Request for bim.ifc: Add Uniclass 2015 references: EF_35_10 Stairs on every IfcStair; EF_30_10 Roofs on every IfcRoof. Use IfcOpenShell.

First a look at what the model holds.

```python
import ifcopenshell

model = ifcopenshell.open("bim.ifc")
print(model.schema)
print("classifications:", [c.Name for c in model.by_type("IfcClassification")])
for ifc_class in ("IfcDoor", "IfcRoof", "IfcStair", "IfcWall", "IfcWindow"):
    print(ifc_class, len(model.by_type(ifc_class)))
```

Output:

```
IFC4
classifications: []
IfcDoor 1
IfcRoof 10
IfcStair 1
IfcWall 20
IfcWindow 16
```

```python
import ifcopenshell
import ifcopenshell.api.classification

model = ifcopenshell.open("bim.ifc")

system = ifcopenshell.api.classification.add_classification(model, classification="Uniclass 2015")

codes = {
    "IfcStair": ("EF_35_10", "Stairs"),
    "IfcRoof": ("EF_30_10", "Roofs"),
}
for ifc_class, (code, name) in codes.items():
    products = model.by_type(ifc_class)
    ifcopenshell.api.classification.add_reference(
        model, products=products, classification=system, identification=code, name=name
    )
    print(code, len(products))

model.write("bim_rev.ifc")
```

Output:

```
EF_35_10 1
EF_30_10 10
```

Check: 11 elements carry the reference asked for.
